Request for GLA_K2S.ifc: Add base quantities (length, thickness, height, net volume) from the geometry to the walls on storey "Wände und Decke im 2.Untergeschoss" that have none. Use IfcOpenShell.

First a look at what the model holds.

```python
import ifcopenshell
import ifcopenshell.util.element
import ifcopenshell.util.unit

model = ifcopenshell.open("GLA_K2S.ifc")
print(model.schema)
for unit_type in ("LENGTHUNIT", "AREAUNIT", "VOLUMEUNIT"):
    print(unit_type, ifcopenshell.util.unit.calculate_unit_scale(model, unit_type))
storey = next(s for s in model.by_type("IfcBuildingStorey") if s.Name == "Wände und Decke im 2.Untergeschoss")
walls = [e for e in ifcopenshell.util.element.get_decomposition(storey) if e.is_a("IfcWall")]
for e in sorted(walls, key=lambda e: e.id()):
    print(e.id(), e.is_a(), e.Name, list(ifcopenshell.util.element.get_psets(e, qtos_only=True)), sep=" | ")
```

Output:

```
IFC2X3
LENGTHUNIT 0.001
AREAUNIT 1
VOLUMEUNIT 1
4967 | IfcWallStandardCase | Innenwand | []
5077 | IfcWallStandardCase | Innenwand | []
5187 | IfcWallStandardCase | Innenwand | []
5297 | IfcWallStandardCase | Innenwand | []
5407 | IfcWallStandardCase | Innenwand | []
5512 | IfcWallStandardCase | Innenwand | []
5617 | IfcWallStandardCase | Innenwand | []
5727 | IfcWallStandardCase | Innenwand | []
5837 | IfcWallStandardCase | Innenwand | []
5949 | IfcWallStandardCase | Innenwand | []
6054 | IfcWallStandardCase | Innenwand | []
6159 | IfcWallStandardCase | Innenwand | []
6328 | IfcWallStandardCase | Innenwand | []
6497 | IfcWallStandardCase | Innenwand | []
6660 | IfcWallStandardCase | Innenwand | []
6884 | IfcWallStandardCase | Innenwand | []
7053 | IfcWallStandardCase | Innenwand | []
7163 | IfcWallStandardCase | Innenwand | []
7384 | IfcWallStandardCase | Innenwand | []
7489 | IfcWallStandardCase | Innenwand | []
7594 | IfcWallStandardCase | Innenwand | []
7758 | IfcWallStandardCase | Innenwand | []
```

```python
import ifcopenshell
import ifcopenshell.api.pset
import ifcopenshell.geom
import ifcopenshell.util.element
import ifcopenshell.util.shape
import ifcopenshell.util.unit

model = ifcopenshell.open("GLA_K2S.ifc")
unit_scale = ifcopenshell.util.unit.calculate_unit_scale(model)
volume_scale = ifcopenshell.util.unit.calculate_unit_scale(model, "VOLUMEUNIT")
settings = ifcopenshell.geom.settings()

storey = next(s for s in model.by_type("IfcBuildingStorey") if s.Name == "Wände und Decke im 2.Untergeschoss")
walls = [e for e in ifcopenshell.util.element.get_decomposition(storey) if e.is_a("IfcWall")]

for e in sorted(walls, key=lambda e: e.id()):
    if ifcopenshell.util.element.get_psets(e, qtos_only=True, should_inherit=False):
        continue
    # Geometry comes back in metres, in the element's own axes.
    shape = ifcopenshell.geom.create_shape(settings, e)
    values = {
        "Length": ifcopenshell.util.shape.get_x(shape.geometry) / unit_scale,
        "Width": ifcopenshell.util.shape.get_y(shape.geometry) / unit_scale,
        "Height": ifcopenshell.util.shape.get_z(shape.geometry) / unit_scale,
        "NetVolume": ifcopenshell.util.shape.get_volume(shape.geometry) / volume_scale,
    }
    qto = ifcopenshell.api.pset.add_qto(model, product=e, name="BaseQuantities")
    ifcopenshell.api.pset.edit_qto(model, qto=qto, properties=values)
    print(e.id(), {k: round(v, 3) for k, v in values.items()})

model.write("GLA_K2S_v2.ifc")
```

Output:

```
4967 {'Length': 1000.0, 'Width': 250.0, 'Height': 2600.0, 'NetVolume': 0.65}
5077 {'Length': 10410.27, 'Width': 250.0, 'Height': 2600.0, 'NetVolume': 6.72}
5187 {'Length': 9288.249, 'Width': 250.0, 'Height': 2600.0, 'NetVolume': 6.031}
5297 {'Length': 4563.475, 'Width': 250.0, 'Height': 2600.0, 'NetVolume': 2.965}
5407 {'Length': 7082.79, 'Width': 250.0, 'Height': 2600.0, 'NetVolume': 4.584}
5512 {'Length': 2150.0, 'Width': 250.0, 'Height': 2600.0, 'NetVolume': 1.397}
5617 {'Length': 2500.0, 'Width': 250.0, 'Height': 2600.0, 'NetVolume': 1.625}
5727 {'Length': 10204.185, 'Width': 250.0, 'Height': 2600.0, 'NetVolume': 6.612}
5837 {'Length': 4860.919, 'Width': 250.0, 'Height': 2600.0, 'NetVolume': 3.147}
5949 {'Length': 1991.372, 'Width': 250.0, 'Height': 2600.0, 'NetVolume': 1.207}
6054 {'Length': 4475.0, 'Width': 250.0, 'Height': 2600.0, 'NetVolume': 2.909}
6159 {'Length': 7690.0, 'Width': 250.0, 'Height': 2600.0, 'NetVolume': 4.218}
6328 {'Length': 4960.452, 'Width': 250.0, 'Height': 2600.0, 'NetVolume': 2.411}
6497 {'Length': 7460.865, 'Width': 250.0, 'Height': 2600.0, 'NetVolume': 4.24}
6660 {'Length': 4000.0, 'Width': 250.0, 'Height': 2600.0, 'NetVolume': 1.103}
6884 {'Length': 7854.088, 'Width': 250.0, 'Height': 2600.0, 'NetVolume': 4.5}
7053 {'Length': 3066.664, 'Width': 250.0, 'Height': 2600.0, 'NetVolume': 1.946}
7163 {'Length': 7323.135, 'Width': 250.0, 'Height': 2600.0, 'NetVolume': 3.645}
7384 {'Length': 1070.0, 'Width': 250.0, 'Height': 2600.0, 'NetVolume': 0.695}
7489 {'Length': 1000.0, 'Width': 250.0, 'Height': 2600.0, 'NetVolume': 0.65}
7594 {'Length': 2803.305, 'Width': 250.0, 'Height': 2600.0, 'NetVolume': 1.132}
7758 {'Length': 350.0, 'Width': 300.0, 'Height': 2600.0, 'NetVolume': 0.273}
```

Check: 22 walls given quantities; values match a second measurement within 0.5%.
